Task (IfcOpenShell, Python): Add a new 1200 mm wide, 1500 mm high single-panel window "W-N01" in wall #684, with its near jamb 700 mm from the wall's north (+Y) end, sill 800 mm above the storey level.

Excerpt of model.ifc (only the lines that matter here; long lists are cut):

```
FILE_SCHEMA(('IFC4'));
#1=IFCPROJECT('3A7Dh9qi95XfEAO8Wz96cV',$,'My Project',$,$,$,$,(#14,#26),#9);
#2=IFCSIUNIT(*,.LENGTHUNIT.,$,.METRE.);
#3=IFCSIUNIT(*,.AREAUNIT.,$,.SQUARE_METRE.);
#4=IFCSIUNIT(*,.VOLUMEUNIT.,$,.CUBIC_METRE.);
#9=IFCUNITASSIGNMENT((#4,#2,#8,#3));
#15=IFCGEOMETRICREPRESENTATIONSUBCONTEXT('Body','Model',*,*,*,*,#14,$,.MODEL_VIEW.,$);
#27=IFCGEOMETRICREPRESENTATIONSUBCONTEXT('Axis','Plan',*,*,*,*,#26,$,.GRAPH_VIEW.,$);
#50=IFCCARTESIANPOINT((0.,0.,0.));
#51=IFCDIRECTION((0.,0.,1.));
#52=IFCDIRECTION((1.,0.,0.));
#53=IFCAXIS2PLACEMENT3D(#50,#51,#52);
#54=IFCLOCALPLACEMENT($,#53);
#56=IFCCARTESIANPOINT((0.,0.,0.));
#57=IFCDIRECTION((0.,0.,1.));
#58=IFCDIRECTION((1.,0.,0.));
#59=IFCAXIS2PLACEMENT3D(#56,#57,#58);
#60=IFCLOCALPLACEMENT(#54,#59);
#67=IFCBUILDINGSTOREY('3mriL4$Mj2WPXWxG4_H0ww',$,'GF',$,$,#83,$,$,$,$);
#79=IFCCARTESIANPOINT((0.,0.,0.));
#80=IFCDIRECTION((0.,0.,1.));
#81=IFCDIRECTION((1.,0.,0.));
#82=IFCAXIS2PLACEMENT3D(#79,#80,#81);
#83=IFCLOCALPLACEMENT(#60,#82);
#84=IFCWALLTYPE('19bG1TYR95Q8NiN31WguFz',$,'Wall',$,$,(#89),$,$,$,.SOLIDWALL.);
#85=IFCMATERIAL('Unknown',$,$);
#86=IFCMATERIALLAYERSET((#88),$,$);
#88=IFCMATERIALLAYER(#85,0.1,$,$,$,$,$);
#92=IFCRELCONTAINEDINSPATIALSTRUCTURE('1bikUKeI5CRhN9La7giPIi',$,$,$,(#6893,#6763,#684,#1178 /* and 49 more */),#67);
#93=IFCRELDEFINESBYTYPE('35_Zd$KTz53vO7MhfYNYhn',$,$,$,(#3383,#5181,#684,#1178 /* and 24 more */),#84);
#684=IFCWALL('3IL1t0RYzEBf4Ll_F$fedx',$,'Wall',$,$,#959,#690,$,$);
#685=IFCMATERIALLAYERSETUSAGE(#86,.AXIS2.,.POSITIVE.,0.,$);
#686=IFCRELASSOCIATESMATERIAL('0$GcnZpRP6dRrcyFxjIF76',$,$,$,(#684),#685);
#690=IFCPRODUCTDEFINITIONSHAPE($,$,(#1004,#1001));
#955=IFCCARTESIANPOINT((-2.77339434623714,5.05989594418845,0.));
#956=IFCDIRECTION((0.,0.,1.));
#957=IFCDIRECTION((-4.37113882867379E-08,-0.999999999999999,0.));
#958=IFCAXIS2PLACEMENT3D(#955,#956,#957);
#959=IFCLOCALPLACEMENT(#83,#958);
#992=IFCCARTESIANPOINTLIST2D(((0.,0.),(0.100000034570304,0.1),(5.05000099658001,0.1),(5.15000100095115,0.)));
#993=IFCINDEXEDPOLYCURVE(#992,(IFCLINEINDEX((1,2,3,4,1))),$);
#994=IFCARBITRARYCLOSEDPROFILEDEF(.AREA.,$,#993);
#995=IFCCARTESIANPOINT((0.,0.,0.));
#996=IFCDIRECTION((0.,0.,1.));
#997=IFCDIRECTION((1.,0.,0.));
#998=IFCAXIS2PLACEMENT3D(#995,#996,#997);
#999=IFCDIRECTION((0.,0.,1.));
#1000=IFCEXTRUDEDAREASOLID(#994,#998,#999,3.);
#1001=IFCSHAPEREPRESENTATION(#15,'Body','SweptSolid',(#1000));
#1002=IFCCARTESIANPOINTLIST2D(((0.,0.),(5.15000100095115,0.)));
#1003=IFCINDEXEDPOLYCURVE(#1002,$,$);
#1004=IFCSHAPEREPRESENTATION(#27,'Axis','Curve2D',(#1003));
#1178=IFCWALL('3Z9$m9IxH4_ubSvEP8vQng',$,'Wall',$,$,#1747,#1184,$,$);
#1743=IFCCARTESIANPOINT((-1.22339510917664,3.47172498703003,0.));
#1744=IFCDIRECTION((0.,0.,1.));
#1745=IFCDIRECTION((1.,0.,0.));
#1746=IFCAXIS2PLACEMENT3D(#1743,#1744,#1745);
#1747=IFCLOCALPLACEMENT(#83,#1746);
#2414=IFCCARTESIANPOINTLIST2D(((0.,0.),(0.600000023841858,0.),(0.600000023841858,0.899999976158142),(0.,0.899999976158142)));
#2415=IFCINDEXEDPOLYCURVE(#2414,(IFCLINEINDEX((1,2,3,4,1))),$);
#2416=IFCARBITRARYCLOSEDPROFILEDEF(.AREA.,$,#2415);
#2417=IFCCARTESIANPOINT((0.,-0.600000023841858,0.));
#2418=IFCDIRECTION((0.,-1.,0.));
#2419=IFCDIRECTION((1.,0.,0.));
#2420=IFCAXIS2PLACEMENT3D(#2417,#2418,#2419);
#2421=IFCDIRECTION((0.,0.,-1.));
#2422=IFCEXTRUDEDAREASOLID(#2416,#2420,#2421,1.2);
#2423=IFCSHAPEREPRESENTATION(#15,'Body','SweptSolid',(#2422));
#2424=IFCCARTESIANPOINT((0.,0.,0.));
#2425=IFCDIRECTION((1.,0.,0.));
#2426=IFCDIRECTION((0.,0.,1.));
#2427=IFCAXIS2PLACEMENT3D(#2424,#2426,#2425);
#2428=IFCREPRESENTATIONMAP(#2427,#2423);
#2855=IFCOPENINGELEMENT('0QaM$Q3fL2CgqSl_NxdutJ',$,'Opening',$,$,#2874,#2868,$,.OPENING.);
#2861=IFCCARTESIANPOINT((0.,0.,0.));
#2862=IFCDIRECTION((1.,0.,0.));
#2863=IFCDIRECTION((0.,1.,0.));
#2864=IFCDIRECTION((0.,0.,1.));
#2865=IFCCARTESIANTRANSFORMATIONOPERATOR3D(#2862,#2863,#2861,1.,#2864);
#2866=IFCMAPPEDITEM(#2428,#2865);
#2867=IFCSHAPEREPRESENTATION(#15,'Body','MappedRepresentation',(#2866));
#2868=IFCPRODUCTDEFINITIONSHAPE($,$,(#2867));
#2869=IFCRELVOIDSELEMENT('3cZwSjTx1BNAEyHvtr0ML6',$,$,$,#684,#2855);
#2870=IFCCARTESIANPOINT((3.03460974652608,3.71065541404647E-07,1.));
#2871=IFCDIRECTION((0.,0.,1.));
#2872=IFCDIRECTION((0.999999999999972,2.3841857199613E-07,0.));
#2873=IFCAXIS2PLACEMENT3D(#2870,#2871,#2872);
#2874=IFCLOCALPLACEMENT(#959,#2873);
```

```python
import numpy as np
import ifcopenshell
import ifcopenshell.api.feature
import ifcopenshell.api.geometry
import ifcopenshell.api.root
import ifcopenshell.api.spatial
import ifcopenshell.geom
import ifcopenshell.util.element
import ifcopenshell.util.placement
import ifcopenshell.util.representation
import ifcopenshell.util.shape
import ifcopenshell.util.unit

model = ifcopenshell.open("model.ifc")
unit_scale = ifcopenshell.util.unit.calculate_unit_scale(model)
settings = ifcopenshell.geom.settings()


def volume(element):
    """Net volume in cubic metres, openings subtracted."""
    shape = ifcopenshell.geom.create_shape(settings, element)
    return ifcopenshell.util.shape.get_volume(shape.geometry)


wall = model.by_id(684)
storey = ifcopenshell.util.element.get_container(wall, ifc_class="IfcBuildingStorey")
context = ifcopenshell.util.representation.get_context(model, "Model", "Body", "MODEL_VIEW")
before = volume(wall)

width, height, from_end, sill = 1.2, 1.5, 0.7, 0.8  # metres

# The wall runs along its own X axis, and the end named is its -X end.
wall_shape = ifcopenshell.geom.create_shape(settings, wall)
x, y, z = ifcopenshell.util.shape.get_vertices(wall_shape.geometry).T
start = x.min() + from_end
face, thickness = float(y.min()), float(y.max() - y.min())
wall_matrix = ifcopenshell.util.placement.get_local_placement(wall.ObjectPlacement)
level = ifcopenshell.util.placement.get_local_placement(storey.ObjectPlacement)[2, 3]


def in_wall(x, y):
    """Placement at x, y metres in the wall's axes, at sill height."""
    matrix = wall_matrix.copy()
    matrix[:, 3] = wall_matrix @ np.array([x / unit_scale, y / unit_scale, 0.0, 1.0])
    matrix[2, 3] = level + sill / unit_scale
    return matrix


# Opening: a box that overshoots both wall faces by 50 mm.
opening = ifcopenshell.api.root.create_entity(model, ifc_class="IfcOpeningElement", predefined_type="OPENING")
box = ifcopenshell.api.geometry.add_wall_representation(
    model, context=context, length=width, height=height, thickness=thickness + 0.1
)
ifcopenshell.api.geometry.assign_representation(model, product=opening, representation=box)
ifcopenshell.api.geometry.edit_object_placement(model, product=opening, matrix=in_wall(start, face - 0.05), is_si=False)
ifcopenshell.api.feature.add_feature(model, feature=opening, element=wall)

window = ifcopenshell.api.root.create_entity(model, ifc_class="IfcWindow", name="W-N01", predefined_type="WINDOW")
window.OverallWidth, window.OverallHeight = width / unit_scale, height / unit_scale
window.PartitioningType = "SINGLE_PANEL"
body = ifcopenshell.api.geometry.add_window_representation(
    model,
    context=context,
    overall_width=window.OverallWidth,
    overall_height=window.OverallHeight,
    partition_type="SINGLE_PANEL",
)
ifcopenshell.api.geometry.assign_representation(model, product=window, representation=body)
ifcopenshell.api.spatial.assign_container(model, products=[window], relating_structure=storey)
ifcopenshell.api.feature.add_filling(model, opening=opening, element=window)

# Centre the window in the wall's thickness.
ifcopenshell.api.geometry.edit_object_placement(model, product=window, matrix=in_wall(start, face), is_si=False)
window_shape = ifcopenshell.geom.create_shape(settings, window)
depth = ifcopenshell.util.shape.get_vertices(window_shape.geometry)[:, 1]
offset = face + thickness / 2 - (depth.min() + depth.max()) / 2
ifcopenshell.api.geometry.edit_object_placement(model, product=window, matrix=in_wall(start, offset), is_si=False)

after = volume(wall)

print(f"wall volume {before:.3f} -> {after:.3f} m3")

model.write("model_rev.ifc")
```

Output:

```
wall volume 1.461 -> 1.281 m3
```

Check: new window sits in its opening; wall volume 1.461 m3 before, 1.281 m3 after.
